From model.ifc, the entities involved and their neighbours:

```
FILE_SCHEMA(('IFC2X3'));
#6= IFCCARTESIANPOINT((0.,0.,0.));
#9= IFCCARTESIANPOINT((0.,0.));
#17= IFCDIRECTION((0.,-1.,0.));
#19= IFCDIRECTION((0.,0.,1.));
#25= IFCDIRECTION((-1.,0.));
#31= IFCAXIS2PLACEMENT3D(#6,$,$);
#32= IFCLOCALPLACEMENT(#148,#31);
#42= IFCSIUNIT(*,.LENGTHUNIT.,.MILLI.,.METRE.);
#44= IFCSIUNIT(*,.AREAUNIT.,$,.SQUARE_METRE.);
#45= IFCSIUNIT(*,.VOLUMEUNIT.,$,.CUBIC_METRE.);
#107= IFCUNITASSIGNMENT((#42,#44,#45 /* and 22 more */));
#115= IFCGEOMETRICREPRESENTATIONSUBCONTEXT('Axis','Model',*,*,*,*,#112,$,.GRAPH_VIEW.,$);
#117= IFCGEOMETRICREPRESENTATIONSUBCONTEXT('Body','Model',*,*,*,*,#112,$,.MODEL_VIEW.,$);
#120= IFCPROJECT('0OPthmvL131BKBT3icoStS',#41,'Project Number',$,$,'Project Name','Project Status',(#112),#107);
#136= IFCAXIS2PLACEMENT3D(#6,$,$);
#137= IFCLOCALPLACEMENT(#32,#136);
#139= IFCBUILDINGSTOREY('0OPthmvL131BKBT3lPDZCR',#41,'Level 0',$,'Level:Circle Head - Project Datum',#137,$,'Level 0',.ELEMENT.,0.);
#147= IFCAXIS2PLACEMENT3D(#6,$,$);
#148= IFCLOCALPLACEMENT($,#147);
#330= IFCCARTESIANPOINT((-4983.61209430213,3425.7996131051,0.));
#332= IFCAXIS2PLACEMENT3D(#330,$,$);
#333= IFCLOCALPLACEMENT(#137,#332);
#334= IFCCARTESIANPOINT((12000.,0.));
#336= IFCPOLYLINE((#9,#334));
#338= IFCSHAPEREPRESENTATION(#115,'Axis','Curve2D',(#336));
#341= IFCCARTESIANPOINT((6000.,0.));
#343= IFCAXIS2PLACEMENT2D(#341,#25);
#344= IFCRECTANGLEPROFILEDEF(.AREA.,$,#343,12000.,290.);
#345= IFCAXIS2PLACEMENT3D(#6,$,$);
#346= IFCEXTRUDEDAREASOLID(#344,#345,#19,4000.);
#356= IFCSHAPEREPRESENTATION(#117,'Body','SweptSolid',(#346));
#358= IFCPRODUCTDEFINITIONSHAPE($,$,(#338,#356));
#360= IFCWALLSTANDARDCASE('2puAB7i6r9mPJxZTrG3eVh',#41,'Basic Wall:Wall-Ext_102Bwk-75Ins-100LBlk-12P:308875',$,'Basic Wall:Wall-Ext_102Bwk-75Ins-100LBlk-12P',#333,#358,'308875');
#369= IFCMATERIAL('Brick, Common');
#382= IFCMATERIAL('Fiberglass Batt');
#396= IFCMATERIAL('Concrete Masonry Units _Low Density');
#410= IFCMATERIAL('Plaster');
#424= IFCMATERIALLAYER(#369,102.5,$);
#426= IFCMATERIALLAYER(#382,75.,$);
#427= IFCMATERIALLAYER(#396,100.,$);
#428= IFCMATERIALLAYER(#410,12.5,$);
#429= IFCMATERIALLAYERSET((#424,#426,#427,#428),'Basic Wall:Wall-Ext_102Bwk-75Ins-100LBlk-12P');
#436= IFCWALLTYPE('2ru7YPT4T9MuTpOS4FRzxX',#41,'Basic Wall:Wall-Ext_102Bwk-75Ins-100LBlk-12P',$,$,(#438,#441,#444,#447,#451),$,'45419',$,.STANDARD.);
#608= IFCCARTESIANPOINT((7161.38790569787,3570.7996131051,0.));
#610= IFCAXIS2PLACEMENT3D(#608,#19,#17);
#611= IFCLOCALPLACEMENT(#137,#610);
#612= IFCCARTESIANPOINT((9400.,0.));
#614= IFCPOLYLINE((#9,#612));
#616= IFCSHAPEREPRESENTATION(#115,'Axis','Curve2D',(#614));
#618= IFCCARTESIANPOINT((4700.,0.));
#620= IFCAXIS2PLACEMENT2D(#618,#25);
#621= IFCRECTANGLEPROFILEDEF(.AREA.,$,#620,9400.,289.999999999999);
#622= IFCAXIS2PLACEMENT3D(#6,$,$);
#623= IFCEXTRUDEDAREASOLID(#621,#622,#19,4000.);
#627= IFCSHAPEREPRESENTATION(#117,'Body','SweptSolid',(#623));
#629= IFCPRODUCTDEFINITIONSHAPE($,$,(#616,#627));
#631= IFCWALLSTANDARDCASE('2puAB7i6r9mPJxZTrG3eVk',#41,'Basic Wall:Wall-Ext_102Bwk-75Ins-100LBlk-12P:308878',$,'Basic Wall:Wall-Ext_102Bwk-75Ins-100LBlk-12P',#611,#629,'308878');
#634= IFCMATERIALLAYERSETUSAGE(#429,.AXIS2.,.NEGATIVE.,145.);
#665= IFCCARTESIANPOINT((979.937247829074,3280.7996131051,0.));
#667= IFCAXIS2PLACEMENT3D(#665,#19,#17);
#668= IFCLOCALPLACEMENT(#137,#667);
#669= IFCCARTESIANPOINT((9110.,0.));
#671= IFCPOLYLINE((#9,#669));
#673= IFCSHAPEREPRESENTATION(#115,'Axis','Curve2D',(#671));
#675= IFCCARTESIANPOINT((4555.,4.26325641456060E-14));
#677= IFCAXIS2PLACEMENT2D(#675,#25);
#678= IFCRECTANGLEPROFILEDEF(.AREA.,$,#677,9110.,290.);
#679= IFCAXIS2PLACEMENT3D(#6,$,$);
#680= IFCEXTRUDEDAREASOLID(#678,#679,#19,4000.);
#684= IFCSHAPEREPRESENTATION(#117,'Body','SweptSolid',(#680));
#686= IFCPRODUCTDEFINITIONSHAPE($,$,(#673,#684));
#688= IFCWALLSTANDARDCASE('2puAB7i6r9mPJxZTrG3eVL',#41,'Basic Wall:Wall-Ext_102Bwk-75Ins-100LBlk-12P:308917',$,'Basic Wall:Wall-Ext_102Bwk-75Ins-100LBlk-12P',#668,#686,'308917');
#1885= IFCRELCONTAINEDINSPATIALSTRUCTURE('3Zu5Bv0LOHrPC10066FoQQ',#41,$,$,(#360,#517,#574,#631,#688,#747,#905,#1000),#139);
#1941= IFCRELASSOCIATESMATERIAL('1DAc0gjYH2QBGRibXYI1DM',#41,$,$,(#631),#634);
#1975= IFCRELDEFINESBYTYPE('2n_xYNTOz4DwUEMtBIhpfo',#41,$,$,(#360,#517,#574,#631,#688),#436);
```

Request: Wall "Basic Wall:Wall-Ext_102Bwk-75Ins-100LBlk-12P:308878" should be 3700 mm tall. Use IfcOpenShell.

```python
import ifcopenshell
import ifcopenshell.geom
import ifcopenshell.util.representation
import ifcopenshell.util.shape
import ifcopenshell.util.unit

model = ifcopenshell.open("model.ifc")
unit_scale = ifcopenshell.util.unit.calculate_unit_scale(model)
settings = ifcopenshell.geom.settings()


def volume(element):
    """Net volume in cubic metres, openings subtracted."""
    shape = ifcopenshell.geom.create_shape(settings, element)
    return ifcopenshell.util.shape.get_volume(shape.geometry)


wall = model.by_guid("2puAB7i6r9mPJxZTrG3eVk")
before = volume(wall)

body = ifcopenshell.util.representation.get_representation(wall, "Model", "Body")
solid = body.Items[0]
old_height = solid.Depth
solid.Depth = 3.7 / unit_scale
after = volume(wall)

print(f"height {old_height:g} -> {solid.Depth:g}, volume {before:.3f} -> {after:.3f} m3")

model.write("model_rev.ifc")
```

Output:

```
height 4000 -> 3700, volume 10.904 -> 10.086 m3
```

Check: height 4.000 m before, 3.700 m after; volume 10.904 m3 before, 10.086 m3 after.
